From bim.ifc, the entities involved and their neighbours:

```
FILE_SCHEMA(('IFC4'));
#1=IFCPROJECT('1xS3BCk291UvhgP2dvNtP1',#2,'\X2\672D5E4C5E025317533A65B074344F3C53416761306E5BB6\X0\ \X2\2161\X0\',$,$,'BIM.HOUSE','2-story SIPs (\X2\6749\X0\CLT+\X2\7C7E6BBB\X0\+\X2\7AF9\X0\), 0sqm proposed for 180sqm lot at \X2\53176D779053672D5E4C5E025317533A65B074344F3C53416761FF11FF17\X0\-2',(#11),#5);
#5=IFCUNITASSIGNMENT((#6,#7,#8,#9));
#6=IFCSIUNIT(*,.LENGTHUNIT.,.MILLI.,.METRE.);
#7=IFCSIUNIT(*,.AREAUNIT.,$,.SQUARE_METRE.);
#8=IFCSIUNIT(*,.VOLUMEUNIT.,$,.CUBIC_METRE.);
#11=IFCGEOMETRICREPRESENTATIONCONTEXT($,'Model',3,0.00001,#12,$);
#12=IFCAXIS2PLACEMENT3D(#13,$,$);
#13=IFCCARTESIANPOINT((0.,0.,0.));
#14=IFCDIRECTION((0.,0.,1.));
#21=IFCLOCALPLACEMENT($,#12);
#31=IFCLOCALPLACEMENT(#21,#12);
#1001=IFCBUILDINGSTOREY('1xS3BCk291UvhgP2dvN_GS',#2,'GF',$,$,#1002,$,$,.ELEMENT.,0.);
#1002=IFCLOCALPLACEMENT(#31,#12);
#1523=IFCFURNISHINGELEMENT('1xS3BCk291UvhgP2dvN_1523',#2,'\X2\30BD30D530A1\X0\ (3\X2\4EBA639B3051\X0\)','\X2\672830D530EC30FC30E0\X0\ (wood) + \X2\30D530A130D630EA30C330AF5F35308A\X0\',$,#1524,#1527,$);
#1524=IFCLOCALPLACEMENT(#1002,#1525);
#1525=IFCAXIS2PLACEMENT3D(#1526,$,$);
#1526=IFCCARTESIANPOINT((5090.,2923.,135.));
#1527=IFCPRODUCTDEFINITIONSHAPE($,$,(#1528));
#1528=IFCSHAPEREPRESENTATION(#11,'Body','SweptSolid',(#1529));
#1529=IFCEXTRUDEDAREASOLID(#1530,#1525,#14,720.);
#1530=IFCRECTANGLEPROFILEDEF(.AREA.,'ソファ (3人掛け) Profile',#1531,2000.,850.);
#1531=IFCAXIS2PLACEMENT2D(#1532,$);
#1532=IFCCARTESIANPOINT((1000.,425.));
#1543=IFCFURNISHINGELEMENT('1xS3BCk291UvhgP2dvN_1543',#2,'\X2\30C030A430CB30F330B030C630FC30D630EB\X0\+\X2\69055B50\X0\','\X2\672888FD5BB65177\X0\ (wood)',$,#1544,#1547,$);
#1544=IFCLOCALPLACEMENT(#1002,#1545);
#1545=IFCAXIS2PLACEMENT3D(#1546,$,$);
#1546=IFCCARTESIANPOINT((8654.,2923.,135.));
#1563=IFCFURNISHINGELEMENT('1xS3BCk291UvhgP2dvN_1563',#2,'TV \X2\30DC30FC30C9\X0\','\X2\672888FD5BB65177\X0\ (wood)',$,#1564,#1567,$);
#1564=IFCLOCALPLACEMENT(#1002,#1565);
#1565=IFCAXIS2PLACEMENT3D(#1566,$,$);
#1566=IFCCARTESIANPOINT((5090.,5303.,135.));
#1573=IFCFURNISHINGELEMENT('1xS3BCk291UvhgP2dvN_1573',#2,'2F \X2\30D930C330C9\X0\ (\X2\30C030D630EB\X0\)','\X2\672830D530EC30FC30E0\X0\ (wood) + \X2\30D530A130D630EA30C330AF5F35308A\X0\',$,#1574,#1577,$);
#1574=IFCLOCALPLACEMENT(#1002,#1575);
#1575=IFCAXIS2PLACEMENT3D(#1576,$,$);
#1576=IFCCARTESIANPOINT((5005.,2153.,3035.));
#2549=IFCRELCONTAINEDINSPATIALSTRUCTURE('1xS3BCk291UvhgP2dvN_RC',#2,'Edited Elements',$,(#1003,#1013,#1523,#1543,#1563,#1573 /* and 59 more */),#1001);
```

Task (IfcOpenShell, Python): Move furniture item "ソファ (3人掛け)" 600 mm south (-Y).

```python
import ifcopenshell
import ifcopenshell.api.geometry
import ifcopenshell.util.placement
import ifcopenshell.util.unit

model = ifcopenshell.open("bim.ifc")
unit_scale = ifcopenshell.util.unit.calculate_unit_scale(model)

item = model.by_id(1523)
matrix = ifcopenshell.util.placement.get_local_placement(item.ObjectPlacement)
matrix[1, 3] -= 0.6 / unit_scale
ifcopenshell.api.geometry.edit_object_placement(model, product=item, matrix=matrix, is_si=False)

print(ifcopenshell.util.placement.get_local_placement(item.ObjectPlacement).round(3) + 0.0)

model.write("bim-out.ifc")
```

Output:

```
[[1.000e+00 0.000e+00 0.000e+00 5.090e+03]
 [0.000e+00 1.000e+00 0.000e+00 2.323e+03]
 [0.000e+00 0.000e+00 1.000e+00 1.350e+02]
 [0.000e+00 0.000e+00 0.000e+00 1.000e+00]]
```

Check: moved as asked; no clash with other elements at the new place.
